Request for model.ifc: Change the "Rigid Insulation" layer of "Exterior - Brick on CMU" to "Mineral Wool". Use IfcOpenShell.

First a look at what the model holds.

```python
import ifcopenshell
import ifcopenshell.util.element

model = ifcopenshell.open("model.ifc")
print(model.schema)
for layer_set in model.by_type("IfcMaterialLayerSet"):
    if layer_set.LayerSetName == "Exterior - Brick on CMU":
        for layer in layer_set.MaterialLayers:
            print(layer.id(), layer.Material and layer.Material.Name, layer.LayerThickness, sep=" | ")
        print(len(ifcopenshell.util.element.get_elements_by_material(model, layer_set)), "elements and types use it")
print(sorted(m.Name for m in model.by_type("IfcMaterial") if m.Name)[:60])
```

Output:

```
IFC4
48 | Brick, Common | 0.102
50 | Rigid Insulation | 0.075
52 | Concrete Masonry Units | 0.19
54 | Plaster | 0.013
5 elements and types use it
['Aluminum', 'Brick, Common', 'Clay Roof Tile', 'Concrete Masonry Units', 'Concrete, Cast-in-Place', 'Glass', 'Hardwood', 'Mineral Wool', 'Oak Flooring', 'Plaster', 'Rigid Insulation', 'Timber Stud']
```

```python
import ifcopenshell
import ifcopenshell.api.material

model = ifcopenshell.open("model.ifc")

layer_set = next(s for s in model.by_type("IfcMaterialLayerSet") if s.LayerSetName == "Exterior - Brick on CMU")
layer = next(l for l in layer_set.MaterialLayers if l.Material and l.Material.Name == "Rigid Insulation")
material = next(m for m in model.by_type("IfcMaterial") if m.Name == "Mineral Wool")

# Point this one layer at the other material; renaming the old one would change it everywhere.
ifcopenshell.api.material.edit_layer(model, layer=layer, attributes={"Name": material.Name}, material=material)

print([l.Material.Name if l.Material else None for l in layer_set.MaterialLayers])

model.write("model-out.ifc")
```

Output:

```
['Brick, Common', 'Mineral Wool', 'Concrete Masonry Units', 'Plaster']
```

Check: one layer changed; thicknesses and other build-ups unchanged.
